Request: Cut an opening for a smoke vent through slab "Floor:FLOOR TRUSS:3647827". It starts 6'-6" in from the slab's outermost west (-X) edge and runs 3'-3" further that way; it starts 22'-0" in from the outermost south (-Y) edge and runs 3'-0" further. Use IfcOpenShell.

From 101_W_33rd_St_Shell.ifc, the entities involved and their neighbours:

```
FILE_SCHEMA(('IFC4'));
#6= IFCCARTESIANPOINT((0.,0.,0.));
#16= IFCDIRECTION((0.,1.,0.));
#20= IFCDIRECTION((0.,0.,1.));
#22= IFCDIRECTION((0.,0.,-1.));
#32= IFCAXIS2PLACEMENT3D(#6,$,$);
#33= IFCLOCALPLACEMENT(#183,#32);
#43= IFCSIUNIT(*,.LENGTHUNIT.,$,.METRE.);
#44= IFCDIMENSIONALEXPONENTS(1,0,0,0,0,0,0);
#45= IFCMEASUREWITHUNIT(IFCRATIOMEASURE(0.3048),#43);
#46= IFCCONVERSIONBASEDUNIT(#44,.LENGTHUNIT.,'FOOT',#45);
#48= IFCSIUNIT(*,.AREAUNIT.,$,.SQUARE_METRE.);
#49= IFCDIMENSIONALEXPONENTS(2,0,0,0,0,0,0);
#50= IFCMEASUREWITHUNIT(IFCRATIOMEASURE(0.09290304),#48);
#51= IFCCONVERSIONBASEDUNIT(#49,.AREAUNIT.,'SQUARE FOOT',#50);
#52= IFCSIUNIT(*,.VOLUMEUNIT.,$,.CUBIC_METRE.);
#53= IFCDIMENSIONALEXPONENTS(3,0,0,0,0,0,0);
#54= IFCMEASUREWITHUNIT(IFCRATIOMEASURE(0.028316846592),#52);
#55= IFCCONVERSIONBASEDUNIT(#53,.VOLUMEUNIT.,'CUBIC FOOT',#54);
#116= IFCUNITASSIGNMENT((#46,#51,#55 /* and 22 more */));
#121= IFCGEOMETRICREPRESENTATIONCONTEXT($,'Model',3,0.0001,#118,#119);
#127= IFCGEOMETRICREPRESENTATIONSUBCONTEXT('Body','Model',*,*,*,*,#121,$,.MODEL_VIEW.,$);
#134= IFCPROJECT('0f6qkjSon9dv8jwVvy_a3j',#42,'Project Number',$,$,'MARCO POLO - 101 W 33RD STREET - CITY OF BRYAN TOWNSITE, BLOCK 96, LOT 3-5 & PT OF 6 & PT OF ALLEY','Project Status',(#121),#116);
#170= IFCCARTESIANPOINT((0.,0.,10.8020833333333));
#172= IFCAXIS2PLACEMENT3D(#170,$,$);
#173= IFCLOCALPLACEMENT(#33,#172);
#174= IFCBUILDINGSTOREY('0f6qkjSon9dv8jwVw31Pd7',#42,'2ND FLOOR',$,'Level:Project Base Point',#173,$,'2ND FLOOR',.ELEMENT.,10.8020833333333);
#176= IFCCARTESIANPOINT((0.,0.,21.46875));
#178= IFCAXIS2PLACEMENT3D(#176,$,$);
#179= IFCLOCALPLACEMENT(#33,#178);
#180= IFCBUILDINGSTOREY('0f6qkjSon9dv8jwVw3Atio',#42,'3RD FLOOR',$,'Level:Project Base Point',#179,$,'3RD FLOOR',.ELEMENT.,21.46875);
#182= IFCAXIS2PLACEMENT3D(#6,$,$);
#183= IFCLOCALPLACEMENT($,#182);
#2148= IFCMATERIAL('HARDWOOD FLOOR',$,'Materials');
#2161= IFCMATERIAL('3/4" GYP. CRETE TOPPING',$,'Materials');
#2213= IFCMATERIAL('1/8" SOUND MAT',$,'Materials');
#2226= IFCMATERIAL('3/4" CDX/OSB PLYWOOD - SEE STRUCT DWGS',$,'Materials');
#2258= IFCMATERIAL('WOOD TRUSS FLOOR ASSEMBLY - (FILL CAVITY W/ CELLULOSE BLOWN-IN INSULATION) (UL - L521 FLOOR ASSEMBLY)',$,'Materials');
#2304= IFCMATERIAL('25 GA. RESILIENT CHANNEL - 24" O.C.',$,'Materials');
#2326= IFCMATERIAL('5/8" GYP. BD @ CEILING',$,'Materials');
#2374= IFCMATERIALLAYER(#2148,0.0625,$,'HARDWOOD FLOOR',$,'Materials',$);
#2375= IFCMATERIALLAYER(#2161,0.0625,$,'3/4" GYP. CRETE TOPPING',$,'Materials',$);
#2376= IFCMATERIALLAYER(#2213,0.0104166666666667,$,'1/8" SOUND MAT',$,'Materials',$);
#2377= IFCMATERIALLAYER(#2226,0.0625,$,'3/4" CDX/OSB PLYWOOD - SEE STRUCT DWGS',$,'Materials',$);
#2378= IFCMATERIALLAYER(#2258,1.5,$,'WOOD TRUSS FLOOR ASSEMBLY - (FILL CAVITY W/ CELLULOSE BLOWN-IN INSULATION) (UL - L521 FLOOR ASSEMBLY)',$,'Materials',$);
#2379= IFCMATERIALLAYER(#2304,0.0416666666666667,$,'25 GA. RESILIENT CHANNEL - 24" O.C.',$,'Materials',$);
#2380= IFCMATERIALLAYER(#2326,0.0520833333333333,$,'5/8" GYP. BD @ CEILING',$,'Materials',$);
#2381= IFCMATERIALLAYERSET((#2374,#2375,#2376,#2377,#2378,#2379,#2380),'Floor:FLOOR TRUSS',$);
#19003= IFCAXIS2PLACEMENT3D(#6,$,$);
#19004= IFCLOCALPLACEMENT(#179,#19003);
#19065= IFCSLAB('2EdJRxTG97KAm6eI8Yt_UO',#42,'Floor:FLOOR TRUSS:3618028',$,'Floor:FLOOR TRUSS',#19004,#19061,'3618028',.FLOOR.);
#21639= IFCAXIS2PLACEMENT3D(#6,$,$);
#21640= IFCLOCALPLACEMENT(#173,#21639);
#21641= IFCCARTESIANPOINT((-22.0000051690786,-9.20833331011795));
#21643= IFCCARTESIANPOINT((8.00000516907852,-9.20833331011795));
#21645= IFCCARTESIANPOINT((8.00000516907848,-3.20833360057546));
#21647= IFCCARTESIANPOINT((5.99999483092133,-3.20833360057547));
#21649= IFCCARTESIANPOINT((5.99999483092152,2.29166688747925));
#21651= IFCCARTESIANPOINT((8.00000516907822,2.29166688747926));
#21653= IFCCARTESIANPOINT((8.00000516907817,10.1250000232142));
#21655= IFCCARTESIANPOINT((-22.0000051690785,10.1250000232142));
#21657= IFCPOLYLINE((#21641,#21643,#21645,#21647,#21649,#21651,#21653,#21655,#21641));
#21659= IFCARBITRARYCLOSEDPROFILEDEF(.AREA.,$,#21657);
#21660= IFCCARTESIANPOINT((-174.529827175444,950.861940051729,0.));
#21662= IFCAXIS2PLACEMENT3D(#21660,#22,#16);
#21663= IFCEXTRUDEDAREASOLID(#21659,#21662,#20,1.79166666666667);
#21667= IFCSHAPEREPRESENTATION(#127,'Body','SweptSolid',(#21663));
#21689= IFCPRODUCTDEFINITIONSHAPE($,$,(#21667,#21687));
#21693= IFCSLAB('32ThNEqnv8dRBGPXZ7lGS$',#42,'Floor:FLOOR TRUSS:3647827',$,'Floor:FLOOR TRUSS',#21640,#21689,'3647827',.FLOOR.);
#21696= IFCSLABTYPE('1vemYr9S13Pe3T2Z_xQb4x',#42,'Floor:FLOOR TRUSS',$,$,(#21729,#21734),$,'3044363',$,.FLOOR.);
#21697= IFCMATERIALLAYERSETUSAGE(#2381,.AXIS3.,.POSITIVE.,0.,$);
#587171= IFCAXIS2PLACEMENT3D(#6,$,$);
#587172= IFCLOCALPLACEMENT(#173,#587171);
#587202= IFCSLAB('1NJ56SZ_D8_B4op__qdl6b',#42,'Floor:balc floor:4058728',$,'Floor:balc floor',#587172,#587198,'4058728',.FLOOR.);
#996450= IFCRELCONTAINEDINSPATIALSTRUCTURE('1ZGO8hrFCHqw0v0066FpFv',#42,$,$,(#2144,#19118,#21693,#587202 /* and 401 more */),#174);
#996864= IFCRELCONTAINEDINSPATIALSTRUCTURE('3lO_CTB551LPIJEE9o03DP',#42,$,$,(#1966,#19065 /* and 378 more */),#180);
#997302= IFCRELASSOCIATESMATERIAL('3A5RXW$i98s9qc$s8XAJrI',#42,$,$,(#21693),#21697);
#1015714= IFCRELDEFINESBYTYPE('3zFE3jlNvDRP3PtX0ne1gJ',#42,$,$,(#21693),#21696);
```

```python
import numpy as np
import ifcopenshell
import ifcopenshell.api.feature
import ifcopenshell.api.geometry
import ifcopenshell.api.root
import ifcopenshell.geom
import ifcopenshell.util.placement
import ifcopenshell.util.representation
import ifcopenshell.util.shape
import ifcopenshell.util.unit

model = ifcopenshell.open("101_W_33rd_St_Shell.ifc")
unit_scale = ifcopenshell.util.unit.calculate_unit_scale(model)
settings = ifcopenshell.geom.settings()


def volume(element):
    """Net volume in cubic metres, openings subtracted."""
    shape = ifcopenshell.geom.create_shape(settings, element)
    return ifcopenshell.util.shape.get_volume(shape.geometry)


slab = model.by_guid("32ThNEqnv8dRBGPXZ7lGS$")
before = volume(slab)

# Extent in the slab's own axes, in metres. The edges named are its -X and -Y sides.
slab_shape = ifcopenshell.geom.create_shape(settings, slab)
vertices = ifcopenshell.util.shape.get_vertices(slab_shape.geometry)
x_min, y_min, bottom = vertices.min(axis=0)
top = vertices[:, 2].max()

opening = ifcopenshell.api.root.create_entity(model, ifc_class="IfcOpeningElement", name="Smoke vent opening", predefined_type="OPENING")
context = ifcopenshell.util.representation.get_context(model, "Model", "Body", "MODEL_VIEW")
width, depth = 0.9906, 0.9144
outline = [(0.0, 0.0), (width, 0.0), (width, depth), (0.0, depth), (0.0, 0.0)]
# Overshoot both faces by 50 mm so the cut is clean.
shape = ifcopenshell.api.geometry.add_slab_representation(
    model, context=context, depth=top - bottom + 0.1, polyline=outline
)
ifcopenshell.api.geometry.assign_representation(model, product=opening, representation=shape)

matrix = ifcopenshell.util.placement.get_local_placement(slab.ObjectPlacement)
matrix[:, 3] = matrix @ np.append(np.array([x_min + 1.9812, y_min + 6.7056, bottom - 0.05]) / unit_scale, 1.0)
ifcopenshell.api.geometry.edit_object_placement(model, product=opening, matrix=matrix, is_si=False)
ifcopenshell.api.feature.add_feature(model, feature=opening, element=slab)

after = volume(slab)

print(f"slab volume {before:.3f} -> {after:.3f} m3")

model.write("101_W_33rd_St_Shell-out.ifc")
```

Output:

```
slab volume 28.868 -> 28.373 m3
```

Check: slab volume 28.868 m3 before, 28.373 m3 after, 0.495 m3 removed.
